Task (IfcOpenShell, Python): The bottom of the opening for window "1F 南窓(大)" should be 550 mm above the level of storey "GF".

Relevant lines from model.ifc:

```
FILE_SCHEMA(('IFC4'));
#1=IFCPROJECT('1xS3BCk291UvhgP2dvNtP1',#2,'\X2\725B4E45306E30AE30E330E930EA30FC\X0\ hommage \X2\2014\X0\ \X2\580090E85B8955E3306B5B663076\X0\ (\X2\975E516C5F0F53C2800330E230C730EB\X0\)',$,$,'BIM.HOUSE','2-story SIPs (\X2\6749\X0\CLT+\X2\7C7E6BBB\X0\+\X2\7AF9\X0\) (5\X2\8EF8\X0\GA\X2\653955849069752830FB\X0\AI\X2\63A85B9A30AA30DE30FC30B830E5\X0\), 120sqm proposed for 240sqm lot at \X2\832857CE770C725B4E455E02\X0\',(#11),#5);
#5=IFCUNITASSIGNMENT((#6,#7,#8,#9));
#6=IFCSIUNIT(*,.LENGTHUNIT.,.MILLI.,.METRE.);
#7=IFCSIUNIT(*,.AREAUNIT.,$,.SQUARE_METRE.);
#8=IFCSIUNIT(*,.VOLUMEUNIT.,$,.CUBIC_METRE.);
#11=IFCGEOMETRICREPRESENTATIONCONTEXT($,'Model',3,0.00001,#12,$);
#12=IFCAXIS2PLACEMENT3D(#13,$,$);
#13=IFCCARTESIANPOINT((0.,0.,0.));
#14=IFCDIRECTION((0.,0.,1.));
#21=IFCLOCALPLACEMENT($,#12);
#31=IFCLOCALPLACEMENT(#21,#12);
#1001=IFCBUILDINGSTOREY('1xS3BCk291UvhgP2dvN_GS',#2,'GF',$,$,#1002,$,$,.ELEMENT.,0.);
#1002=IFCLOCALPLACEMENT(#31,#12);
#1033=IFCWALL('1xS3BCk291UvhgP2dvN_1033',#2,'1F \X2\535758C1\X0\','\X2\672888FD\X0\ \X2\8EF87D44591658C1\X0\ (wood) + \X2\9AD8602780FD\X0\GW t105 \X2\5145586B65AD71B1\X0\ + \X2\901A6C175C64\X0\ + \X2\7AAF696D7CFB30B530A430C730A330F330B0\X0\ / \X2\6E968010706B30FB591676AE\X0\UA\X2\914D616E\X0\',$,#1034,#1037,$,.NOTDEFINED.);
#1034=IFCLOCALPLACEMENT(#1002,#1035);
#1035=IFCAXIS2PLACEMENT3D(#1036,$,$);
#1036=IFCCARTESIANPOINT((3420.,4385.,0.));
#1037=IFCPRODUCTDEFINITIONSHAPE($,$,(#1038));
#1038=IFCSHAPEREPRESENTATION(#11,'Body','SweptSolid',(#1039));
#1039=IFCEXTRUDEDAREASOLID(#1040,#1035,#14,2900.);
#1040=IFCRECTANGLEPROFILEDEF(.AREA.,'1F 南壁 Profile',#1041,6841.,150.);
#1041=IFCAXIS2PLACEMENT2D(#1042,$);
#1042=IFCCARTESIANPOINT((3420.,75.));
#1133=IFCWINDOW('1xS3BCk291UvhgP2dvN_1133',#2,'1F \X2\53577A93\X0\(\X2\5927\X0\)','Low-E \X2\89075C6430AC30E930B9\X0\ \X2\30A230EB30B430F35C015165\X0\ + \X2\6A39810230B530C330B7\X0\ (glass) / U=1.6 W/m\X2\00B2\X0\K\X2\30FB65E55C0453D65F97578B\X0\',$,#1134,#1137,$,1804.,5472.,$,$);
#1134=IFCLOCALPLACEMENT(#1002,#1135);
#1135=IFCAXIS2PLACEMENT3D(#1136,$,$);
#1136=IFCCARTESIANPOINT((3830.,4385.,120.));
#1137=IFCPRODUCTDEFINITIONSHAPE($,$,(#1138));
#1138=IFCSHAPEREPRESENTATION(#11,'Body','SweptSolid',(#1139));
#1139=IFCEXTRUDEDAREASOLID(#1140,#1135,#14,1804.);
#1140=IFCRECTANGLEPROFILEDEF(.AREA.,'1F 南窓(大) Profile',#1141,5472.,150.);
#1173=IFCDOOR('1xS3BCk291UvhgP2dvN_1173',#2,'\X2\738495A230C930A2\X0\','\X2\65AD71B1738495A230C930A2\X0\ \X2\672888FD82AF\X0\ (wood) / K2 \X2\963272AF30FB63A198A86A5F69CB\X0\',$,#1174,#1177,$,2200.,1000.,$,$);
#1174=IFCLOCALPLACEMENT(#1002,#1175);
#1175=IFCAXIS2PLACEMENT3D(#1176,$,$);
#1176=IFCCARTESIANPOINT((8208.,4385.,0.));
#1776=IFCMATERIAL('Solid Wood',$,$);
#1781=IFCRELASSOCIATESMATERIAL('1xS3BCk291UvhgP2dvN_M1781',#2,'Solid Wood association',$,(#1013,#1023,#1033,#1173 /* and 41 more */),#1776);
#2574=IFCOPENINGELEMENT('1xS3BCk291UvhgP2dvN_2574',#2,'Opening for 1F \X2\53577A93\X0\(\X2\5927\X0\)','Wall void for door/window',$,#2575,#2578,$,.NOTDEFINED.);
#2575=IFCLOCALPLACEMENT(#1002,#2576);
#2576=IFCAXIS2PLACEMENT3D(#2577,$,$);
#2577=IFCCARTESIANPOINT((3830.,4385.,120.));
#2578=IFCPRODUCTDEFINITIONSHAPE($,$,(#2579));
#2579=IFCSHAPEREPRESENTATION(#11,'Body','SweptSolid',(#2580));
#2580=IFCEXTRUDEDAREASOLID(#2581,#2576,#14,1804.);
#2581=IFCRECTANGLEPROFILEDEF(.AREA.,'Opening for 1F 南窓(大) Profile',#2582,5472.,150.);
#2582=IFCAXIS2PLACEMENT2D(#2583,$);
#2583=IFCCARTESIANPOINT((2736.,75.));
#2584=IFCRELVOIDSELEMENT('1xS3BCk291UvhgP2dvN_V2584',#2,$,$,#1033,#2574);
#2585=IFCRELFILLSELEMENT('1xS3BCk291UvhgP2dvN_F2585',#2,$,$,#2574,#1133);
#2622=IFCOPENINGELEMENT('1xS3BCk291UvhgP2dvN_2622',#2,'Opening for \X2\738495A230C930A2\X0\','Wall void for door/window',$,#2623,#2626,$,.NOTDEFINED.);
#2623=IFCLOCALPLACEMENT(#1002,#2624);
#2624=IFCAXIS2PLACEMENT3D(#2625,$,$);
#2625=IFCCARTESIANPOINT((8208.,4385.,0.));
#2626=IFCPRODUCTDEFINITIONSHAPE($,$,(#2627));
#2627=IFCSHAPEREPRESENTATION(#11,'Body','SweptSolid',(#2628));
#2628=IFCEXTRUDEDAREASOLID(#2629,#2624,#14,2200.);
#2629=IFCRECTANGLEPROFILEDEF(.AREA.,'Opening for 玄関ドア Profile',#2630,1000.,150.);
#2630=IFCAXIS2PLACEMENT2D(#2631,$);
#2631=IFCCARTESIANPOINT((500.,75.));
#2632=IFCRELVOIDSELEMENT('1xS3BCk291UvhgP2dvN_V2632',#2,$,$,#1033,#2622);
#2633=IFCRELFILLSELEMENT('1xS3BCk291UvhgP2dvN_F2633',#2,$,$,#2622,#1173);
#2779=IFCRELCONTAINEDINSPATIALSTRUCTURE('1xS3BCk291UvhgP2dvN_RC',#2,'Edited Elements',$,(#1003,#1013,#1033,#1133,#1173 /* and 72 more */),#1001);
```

```python
import numpy as np
import ifcopenshell
import ifcopenshell.api.geometry
import ifcopenshell.geom
import ifcopenshell.util.element
import ifcopenshell.util.placement
import ifcopenshell.util.shape
import ifcopenshell.util.unit

model = ifcopenshell.open("model.ifc")
unit_scale = ifcopenshell.util.unit.calculate_unit_scale(model)

window = model.by_id(1133)
opening = window.FillsVoids[0].RelatingOpeningElement
storey = ifcopenshell.util.element.get_container(window, ifc_class="IfcBuildingStorey")
level = ifcopenshell.util.placement.get_local_placement(storey.ObjectPlacement)[2, 3]

# The opening's origin need not be at the sill, so measure its lowest point.
shape = ifcopenshell.geom.create_shape(ifcopenshell.geom.settings(), opening)
bottom = ifcopenshell.util.shape.get_shape_bottom_elevation(shape, shape.geometry) / unit_scale
dz = level + 0.55 / unit_scale - bottom

shift = np.array([0.0, 0.0, dz])
# The window is not placed relative to its opening, so move both.
for product in (opening, window):
    matrix = ifcopenshell.util.placement.get_local_placement(product.ObjectPlacement)
    matrix[:3, 3] += shift
    ifcopenshell.api.geometry.edit_object_placement(model, product=product, matrix=matrix, is_si=False)

print(f"moved by {dz * unit_scale:+.3f} m")

model.write("model_v2.ifc")
```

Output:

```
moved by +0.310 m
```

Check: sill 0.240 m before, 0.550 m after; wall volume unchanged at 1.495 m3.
